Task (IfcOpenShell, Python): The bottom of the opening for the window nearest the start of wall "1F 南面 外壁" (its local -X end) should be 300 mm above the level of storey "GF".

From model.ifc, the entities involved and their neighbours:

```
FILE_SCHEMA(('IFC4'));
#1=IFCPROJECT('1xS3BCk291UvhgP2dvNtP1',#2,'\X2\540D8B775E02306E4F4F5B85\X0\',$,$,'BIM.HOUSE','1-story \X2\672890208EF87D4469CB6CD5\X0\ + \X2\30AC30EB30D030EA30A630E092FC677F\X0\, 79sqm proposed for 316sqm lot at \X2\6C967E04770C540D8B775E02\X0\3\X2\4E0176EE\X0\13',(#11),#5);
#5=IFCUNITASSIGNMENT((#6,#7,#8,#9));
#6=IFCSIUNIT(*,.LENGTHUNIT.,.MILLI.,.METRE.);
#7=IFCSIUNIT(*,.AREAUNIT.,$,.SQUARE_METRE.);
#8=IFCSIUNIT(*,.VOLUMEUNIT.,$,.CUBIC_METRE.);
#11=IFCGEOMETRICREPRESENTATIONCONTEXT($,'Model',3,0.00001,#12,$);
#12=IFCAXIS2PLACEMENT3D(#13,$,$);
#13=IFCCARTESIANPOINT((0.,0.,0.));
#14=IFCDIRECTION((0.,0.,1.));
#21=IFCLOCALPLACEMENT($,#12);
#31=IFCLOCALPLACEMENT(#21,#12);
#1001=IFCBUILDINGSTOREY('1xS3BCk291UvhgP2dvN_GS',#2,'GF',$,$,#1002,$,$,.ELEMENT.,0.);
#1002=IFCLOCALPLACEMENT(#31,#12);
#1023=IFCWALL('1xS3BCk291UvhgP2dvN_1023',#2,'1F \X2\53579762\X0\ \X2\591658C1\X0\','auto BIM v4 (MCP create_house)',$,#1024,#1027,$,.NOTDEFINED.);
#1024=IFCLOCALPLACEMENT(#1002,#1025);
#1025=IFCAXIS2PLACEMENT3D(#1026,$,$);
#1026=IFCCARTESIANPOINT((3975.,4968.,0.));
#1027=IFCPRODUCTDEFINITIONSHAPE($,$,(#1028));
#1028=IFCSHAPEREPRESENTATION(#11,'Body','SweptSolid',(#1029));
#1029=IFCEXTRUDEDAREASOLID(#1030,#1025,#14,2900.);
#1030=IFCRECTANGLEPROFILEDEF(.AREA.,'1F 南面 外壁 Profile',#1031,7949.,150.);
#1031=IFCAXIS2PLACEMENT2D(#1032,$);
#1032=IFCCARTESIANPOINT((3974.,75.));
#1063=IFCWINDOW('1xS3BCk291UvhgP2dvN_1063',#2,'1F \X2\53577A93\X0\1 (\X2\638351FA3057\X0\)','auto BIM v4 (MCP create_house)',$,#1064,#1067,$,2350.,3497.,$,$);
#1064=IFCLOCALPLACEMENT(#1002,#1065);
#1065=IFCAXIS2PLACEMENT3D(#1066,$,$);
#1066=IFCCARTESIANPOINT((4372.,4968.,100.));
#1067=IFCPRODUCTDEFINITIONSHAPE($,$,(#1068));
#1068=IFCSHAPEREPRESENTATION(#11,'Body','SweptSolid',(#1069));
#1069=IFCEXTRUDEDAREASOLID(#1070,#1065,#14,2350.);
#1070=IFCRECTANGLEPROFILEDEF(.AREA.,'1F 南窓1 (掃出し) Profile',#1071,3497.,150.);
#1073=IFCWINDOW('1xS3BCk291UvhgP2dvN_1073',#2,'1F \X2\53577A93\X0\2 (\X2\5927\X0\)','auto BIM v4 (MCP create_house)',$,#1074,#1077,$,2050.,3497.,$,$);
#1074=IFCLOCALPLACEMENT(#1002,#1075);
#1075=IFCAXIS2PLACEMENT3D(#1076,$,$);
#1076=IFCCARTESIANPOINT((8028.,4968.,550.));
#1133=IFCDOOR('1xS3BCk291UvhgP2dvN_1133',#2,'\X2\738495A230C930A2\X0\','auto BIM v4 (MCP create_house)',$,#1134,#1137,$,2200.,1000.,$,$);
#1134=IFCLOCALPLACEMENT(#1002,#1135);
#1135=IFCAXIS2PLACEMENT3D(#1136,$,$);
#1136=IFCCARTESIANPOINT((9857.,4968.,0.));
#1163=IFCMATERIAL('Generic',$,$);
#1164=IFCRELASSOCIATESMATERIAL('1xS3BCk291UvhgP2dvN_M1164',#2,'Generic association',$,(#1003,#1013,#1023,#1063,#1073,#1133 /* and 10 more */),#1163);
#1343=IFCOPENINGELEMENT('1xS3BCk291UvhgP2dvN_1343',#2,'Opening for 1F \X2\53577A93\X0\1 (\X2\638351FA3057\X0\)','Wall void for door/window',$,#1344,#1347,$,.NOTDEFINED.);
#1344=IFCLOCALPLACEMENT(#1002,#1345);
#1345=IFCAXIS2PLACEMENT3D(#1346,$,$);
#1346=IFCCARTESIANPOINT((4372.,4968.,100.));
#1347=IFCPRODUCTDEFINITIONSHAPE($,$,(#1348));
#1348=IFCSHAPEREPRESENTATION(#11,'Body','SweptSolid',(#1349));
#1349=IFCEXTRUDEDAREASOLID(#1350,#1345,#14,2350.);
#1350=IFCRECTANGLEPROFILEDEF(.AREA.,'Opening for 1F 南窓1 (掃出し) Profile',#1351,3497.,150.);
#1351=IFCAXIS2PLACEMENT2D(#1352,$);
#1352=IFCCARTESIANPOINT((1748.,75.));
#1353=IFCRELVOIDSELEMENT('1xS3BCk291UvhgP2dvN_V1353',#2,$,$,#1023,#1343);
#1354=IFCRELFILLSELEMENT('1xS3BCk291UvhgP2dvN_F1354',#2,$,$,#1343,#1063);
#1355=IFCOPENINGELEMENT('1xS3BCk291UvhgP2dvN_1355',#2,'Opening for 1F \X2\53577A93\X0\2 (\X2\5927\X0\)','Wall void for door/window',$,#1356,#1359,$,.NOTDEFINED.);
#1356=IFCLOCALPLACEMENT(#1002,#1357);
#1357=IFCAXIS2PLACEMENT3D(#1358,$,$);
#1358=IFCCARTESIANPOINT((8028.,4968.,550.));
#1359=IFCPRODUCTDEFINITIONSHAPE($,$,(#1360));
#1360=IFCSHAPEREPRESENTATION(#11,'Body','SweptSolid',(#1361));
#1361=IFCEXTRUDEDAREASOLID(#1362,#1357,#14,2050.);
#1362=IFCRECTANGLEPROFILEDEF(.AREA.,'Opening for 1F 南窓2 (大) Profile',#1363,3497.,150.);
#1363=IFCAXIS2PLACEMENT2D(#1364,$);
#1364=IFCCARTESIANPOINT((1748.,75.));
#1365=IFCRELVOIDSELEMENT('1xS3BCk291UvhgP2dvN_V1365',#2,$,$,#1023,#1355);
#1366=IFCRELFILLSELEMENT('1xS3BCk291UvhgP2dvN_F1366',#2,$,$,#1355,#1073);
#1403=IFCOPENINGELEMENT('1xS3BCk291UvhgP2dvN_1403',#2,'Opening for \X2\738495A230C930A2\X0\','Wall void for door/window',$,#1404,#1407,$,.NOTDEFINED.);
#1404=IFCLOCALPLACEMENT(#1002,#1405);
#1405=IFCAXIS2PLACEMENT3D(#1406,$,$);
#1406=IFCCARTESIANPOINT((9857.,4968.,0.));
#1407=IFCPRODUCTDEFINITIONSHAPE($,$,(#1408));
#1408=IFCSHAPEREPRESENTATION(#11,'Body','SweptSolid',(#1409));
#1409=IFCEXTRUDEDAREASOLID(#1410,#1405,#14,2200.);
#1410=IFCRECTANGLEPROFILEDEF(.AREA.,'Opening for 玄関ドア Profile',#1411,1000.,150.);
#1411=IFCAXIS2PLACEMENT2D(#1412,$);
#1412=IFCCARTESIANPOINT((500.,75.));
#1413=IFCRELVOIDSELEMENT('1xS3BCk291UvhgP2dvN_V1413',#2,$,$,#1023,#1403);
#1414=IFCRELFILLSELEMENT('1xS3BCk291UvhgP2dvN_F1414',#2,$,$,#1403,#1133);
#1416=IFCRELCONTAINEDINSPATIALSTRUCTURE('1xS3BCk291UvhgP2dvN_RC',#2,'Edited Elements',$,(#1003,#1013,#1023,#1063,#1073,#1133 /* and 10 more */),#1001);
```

```python
import numpy as np
import ifcopenshell
import ifcopenshell.api.geometry
import ifcopenshell.geom
import ifcopenshell.util.element
import ifcopenshell.util.placement
import ifcopenshell.util.shape
import ifcopenshell.util.unit

model = ifcopenshell.open("model.ifc")
unit_scale = ifcopenshell.util.unit.calculate_unit_scale(model)

window = model.by_guid("1xS3BCk291UvhgP2dvN_1063")
opening = window.FillsVoids[0].RelatingOpeningElement
storey = ifcopenshell.util.element.get_container(window, ifc_class="IfcBuildingStorey")
level = ifcopenshell.util.placement.get_local_placement(storey.ObjectPlacement)[2, 3]

# The opening's origin need not be at the sill, so measure its lowest point.
shape = ifcopenshell.geom.create_shape(ifcopenshell.geom.settings(), opening)
bottom = ifcopenshell.util.shape.get_shape_bottom_elevation(shape, shape.geometry) / unit_scale
dz = level + 0.3 / unit_scale - bottom

shift = np.array([0.0, 0.0, dz])
# The window is not placed relative to its opening, so move both.
for product in (opening, window):
    matrix = ifcopenshell.util.placement.get_local_placement(product.ObjectPlacement)
    matrix[:3, 3] += shift
    ifcopenshell.api.geometry.edit_object_placement(model, product=product, matrix=matrix, is_si=False)

print(f"moved by {dz * unit_scale:+.3f} m")

model.write("model-out.ifc")
```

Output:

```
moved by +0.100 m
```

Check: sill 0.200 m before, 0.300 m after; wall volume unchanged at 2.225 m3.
